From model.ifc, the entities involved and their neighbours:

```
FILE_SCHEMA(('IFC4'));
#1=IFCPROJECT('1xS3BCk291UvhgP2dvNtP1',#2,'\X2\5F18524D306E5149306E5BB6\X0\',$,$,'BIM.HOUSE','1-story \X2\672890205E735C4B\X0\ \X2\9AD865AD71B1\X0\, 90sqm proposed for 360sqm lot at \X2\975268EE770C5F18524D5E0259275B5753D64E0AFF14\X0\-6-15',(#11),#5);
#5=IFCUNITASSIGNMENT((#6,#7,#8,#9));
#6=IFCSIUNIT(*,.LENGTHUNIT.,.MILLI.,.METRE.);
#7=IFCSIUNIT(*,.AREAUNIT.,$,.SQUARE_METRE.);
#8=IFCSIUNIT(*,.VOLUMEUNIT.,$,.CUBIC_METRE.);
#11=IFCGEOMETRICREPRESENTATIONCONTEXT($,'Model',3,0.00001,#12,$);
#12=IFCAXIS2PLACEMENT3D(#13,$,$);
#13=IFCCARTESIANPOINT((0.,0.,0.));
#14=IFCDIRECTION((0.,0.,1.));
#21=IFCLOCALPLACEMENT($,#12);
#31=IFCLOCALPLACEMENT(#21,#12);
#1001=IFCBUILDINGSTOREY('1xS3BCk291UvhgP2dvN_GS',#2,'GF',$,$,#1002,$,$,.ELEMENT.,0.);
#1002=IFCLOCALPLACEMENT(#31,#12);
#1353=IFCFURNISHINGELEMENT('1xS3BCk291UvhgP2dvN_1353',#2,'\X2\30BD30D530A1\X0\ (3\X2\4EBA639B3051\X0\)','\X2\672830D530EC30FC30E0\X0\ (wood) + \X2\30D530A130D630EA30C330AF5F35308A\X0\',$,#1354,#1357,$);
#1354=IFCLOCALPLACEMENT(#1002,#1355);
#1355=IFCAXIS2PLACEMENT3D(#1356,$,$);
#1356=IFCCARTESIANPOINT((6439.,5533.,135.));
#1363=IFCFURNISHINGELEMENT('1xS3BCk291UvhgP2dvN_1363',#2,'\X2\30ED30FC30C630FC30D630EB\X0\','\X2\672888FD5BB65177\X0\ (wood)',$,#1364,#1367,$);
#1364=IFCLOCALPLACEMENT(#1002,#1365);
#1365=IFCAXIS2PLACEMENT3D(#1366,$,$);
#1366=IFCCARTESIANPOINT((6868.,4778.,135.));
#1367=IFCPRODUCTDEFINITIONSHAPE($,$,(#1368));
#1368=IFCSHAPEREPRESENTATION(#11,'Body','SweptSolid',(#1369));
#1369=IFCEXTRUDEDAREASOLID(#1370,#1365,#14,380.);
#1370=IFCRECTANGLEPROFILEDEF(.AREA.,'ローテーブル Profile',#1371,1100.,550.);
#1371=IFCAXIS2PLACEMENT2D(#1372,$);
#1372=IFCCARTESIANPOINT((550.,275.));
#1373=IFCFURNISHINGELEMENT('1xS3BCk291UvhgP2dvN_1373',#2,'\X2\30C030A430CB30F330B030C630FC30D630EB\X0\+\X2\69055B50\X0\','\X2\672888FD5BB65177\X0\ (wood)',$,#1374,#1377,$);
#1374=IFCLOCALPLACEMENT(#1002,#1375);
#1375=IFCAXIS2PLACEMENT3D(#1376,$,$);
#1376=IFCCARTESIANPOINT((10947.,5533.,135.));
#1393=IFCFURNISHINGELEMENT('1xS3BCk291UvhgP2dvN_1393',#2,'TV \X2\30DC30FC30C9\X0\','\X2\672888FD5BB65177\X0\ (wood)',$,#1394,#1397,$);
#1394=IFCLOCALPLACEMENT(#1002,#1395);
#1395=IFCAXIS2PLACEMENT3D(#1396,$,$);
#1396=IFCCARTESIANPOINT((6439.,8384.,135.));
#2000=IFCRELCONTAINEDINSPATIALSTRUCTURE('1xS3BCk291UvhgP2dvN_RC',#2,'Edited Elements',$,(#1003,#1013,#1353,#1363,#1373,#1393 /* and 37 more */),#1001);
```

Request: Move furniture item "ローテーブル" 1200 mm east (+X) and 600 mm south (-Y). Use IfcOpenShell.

```python
import ifcopenshell
import ifcopenshell.api.geometry
import ifcopenshell.util.placement

model = ifcopenshell.open("model.ifc")

item = model.by_guid("1xS3BCk291UvhgP2dvN_1363")
matrix = ifcopenshell.util.placement.get_local_placement(item.ObjectPlacement)
matrix[0, 3] += 1200.0
matrix[1, 3] -= 600.0
ifcopenshell.api.geometry.edit_object_placement(model, product=item, matrix=matrix, is_si=False)

print(ifcopenshell.util.placement.get_local_placement(item.ObjectPlacement).round(3) + 0.0)

model.write("model_updated.ifc")
```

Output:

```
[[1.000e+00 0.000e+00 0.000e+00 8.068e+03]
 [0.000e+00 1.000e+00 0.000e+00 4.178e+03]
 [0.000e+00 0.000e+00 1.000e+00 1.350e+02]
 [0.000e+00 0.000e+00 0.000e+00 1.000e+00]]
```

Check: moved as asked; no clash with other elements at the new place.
